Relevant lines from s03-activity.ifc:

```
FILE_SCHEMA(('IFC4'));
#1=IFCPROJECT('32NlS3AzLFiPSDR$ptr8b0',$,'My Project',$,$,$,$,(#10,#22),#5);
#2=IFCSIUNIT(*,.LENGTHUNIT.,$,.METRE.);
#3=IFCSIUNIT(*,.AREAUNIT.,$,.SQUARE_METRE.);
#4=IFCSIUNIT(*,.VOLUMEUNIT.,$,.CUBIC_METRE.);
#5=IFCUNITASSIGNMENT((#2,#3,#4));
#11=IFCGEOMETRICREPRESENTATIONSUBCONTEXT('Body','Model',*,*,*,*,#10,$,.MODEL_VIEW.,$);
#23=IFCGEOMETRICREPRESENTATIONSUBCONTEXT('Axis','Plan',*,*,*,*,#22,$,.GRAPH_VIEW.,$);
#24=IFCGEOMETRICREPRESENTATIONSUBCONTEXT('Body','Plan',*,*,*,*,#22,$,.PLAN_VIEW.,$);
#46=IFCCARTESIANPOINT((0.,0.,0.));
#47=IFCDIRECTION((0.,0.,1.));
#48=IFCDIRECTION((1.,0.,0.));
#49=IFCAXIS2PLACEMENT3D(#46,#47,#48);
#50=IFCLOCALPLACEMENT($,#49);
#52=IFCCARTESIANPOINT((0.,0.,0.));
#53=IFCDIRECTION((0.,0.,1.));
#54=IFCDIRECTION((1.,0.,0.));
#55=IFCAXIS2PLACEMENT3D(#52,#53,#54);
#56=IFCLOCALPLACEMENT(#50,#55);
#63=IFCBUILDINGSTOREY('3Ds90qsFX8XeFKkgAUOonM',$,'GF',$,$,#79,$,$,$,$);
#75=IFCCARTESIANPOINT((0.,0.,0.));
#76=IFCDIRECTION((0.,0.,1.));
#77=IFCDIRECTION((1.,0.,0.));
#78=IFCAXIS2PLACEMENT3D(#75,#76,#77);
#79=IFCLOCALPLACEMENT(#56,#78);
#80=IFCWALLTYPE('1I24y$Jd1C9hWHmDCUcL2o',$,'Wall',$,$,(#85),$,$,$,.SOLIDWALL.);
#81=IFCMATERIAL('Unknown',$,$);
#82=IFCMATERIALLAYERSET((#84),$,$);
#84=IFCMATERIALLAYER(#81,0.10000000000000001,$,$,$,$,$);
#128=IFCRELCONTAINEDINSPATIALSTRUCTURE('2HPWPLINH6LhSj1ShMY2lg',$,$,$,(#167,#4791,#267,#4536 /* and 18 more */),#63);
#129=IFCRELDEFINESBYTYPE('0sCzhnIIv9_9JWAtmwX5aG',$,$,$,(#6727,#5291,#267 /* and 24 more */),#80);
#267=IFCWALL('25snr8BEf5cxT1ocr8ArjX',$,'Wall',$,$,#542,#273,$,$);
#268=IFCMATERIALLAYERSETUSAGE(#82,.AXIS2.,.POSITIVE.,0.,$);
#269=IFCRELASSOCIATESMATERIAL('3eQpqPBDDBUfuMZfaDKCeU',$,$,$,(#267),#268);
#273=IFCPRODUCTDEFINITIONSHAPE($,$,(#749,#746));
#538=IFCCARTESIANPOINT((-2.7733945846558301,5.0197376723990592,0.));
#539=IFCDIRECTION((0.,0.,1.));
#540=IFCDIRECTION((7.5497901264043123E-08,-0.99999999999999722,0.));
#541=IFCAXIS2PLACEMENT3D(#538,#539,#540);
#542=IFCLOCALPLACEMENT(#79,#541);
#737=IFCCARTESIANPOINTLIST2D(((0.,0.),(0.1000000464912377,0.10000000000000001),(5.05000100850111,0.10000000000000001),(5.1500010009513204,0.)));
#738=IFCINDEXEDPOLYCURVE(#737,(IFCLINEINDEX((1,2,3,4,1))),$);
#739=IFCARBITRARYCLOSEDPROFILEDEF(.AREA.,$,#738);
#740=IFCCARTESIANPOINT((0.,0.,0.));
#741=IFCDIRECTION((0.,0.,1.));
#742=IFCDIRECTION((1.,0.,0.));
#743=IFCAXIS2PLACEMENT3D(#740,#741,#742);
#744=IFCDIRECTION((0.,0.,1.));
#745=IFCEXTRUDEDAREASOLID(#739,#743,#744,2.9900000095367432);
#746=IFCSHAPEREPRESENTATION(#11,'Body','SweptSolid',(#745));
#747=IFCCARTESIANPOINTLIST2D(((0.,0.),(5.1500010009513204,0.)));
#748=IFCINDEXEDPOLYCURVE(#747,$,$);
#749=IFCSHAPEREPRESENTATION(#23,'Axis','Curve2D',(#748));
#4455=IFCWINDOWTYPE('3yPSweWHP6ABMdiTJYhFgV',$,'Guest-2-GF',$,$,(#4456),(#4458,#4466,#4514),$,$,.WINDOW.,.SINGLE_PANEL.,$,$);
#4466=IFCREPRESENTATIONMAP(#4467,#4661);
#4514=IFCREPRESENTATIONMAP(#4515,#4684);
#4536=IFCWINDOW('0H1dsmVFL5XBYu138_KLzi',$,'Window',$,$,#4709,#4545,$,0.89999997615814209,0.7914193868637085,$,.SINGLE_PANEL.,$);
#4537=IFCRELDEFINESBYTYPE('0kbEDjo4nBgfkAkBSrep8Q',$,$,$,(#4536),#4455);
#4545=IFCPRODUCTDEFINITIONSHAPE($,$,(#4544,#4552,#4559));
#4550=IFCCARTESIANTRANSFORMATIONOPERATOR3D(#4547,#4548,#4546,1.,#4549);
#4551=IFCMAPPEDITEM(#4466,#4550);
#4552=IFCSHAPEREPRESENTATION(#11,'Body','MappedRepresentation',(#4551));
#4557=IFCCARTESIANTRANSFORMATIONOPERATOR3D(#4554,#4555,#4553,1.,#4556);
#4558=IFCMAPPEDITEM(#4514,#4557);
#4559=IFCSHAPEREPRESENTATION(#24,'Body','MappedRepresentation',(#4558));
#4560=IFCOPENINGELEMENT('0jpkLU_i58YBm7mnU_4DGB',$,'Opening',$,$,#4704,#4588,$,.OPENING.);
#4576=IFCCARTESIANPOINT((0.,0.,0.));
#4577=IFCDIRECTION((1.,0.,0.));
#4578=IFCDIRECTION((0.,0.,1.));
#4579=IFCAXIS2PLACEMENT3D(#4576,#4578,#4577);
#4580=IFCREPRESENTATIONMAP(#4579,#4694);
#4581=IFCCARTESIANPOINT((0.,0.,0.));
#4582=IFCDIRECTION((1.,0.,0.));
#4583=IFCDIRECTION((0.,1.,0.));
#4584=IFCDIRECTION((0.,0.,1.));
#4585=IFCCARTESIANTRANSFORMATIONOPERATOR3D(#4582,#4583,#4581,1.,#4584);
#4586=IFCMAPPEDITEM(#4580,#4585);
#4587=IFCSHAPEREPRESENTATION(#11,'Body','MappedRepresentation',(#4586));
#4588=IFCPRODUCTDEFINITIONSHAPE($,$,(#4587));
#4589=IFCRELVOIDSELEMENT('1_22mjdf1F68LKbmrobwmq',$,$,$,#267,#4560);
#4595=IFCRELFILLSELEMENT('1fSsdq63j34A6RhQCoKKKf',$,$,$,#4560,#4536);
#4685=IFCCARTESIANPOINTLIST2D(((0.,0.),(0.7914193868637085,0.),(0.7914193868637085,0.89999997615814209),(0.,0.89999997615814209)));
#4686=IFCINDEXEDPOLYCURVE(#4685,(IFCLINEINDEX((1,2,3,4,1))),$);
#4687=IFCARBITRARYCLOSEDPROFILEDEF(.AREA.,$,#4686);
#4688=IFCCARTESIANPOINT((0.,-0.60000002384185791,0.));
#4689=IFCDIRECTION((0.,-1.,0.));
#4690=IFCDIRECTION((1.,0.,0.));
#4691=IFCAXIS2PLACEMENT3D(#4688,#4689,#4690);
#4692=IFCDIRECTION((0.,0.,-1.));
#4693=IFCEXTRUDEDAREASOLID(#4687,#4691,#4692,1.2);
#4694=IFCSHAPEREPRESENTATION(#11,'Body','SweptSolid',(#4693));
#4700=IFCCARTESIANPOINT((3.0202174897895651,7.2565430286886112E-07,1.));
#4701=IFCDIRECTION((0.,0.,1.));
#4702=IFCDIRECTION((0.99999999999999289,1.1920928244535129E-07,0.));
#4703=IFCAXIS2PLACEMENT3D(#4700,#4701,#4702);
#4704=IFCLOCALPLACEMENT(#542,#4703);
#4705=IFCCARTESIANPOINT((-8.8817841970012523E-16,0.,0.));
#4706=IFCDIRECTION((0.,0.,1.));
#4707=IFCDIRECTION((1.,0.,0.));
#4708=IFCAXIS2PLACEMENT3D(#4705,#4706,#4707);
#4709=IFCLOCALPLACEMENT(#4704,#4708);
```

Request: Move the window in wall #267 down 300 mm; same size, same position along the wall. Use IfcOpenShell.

```python
import numpy as np
import ifcopenshell
import ifcopenshell.api.geometry
import ifcopenshell.util.placement
import ifcopenshell.util.unit

model = ifcopenshell.open("s03-activity.ifc")
unit_scale = ifcopenshell.util.unit.calculate_unit_scale(model)

window = model.by_guid("0H1dsmVFL5XBYu138_KLzi")
opening = window.FillsVoids[0].RelatingOpeningElement
dz = -0.3 / unit_scale

shift = np.array([0.0, 0.0, dz])
# The window is placed relative to its opening, so it follows when the opening moves.
matrix = ifcopenshell.util.placement.get_local_placement(opening.ObjectPlacement)
matrix[:3, 3] += shift
ifcopenshell.api.geometry.edit_object_placement(
    model, product=opening, matrix=matrix, is_si=False, should_transform_children=True
)

print(f"moved by {dz * unit_scale:+.3f} m")

model.write("s03-activity_v2.ifc")
```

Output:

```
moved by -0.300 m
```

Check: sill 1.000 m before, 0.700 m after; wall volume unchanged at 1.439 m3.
